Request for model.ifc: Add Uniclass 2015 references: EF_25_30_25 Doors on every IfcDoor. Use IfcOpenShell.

First a look at what the model holds.

```python
import ifcopenshell

model = ifcopenshell.open("model.ifc")
print(model.schema)
print("classifications:", [c.Name for c in model.by_type("IfcClassification")])
for ifc_class in ("IfcDoor", "IfcRoof", "IfcStair", "IfcWall", "IfcWindow"):
    print(ifc_class, len(model.by_type(ifc_class)))
```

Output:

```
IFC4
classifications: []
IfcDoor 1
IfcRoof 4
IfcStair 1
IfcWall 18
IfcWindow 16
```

```python
import ifcopenshell
import ifcopenshell.api.classification

model = ifcopenshell.open("model.ifc")

system = ifcopenshell.api.classification.add_classification(model, classification="Uniclass 2015")

codes = {
    "IfcDoor": ("EF_25_30_25", "Doors"),
}
for ifc_class, (code, name) in codes.items():
    products = model.by_type(ifc_class)
    ifcopenshell.api.classification.add_reference(
        model, products=products, classification=system, identification=code, name=name
    )
    print(code, len(products))

model.write("model_v2.ifc")
```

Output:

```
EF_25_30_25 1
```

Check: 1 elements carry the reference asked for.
